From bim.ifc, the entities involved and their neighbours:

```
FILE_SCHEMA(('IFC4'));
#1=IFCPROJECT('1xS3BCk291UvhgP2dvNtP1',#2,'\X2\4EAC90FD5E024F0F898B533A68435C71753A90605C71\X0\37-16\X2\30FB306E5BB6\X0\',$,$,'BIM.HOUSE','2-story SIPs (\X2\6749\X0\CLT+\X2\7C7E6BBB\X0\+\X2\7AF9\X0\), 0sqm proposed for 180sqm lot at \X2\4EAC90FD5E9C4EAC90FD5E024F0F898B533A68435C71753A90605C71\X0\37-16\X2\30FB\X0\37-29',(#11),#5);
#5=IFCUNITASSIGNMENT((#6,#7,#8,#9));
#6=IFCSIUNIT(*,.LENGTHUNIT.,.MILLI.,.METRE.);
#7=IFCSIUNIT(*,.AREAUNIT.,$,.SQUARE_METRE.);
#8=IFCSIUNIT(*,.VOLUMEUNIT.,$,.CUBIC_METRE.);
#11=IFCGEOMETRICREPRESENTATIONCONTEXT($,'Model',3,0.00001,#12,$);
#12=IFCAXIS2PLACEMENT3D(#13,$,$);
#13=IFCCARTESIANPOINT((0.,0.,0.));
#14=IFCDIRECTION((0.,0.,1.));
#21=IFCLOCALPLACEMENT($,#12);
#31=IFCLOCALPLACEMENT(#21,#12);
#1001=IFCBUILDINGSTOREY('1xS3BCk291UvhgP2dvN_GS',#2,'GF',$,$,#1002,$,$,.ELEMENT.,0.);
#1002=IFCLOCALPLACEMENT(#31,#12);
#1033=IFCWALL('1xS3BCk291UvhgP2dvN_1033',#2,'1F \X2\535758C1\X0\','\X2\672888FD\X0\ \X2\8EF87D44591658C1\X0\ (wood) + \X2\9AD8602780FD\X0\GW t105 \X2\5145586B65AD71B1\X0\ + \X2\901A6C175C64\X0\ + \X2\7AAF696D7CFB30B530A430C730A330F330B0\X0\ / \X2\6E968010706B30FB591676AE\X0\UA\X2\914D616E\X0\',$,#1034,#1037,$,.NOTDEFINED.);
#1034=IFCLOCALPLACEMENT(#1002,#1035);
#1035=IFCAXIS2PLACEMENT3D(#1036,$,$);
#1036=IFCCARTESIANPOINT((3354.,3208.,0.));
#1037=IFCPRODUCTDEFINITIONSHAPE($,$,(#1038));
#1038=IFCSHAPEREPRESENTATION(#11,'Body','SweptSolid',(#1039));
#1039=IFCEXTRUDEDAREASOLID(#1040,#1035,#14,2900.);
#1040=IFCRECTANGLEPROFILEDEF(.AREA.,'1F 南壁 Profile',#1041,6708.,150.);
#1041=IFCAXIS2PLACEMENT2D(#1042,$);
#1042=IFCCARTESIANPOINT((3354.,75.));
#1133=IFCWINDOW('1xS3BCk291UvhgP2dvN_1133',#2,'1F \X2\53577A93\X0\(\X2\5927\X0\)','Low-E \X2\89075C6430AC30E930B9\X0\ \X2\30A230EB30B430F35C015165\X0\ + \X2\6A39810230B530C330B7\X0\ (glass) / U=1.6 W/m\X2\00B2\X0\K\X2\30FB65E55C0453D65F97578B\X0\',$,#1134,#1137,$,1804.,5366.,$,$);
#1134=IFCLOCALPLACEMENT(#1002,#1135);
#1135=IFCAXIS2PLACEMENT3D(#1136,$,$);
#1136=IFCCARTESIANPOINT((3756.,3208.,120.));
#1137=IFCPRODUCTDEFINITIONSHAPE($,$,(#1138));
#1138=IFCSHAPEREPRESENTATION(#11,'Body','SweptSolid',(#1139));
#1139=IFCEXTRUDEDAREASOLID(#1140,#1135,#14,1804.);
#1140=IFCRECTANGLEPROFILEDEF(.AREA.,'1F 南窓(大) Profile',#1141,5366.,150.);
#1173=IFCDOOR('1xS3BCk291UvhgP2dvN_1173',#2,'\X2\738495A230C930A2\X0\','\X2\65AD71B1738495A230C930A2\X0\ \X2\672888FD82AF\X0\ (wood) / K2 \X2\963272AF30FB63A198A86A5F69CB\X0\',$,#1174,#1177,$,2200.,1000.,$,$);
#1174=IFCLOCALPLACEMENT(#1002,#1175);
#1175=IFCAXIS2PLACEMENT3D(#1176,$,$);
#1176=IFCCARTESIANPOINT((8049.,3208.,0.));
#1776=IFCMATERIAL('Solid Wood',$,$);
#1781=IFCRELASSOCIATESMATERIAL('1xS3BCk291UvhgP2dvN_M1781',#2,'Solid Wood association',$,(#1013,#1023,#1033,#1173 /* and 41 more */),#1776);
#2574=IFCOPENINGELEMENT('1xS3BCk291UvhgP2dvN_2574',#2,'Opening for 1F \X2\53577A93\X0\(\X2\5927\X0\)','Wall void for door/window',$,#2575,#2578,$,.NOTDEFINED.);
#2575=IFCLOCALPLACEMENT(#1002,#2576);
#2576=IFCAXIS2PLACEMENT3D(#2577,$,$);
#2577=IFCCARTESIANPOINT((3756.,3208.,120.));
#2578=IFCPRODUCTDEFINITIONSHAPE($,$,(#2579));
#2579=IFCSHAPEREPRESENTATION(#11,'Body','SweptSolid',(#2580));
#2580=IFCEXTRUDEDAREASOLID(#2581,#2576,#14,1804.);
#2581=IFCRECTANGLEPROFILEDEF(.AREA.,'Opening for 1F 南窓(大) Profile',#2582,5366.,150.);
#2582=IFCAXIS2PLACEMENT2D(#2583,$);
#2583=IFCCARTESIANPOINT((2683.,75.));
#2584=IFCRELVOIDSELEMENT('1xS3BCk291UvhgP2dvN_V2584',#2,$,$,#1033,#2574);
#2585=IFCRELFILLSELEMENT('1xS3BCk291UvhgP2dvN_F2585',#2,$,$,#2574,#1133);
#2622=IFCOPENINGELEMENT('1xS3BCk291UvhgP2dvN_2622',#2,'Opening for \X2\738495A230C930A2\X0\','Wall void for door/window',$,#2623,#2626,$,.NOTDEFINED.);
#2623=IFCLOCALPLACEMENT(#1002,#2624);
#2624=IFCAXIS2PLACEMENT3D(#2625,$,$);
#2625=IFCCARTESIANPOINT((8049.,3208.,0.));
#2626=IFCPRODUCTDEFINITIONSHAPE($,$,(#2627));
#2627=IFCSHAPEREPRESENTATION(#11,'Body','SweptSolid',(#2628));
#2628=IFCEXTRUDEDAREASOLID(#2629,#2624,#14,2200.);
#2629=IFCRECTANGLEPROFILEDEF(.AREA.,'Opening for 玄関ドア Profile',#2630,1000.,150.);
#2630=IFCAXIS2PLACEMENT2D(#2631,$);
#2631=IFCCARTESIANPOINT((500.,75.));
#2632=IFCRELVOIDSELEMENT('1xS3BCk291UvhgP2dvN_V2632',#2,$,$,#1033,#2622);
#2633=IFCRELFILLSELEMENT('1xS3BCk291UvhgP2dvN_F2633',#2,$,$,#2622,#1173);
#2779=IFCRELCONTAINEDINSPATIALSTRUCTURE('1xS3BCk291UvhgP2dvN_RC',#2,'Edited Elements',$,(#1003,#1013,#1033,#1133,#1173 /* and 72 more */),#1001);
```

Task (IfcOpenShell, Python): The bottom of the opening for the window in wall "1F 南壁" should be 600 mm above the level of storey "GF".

```python
import numpy as np
import ifcopenshell
import ifcopenshell.api.geometry
import ifcopenshell.geom
import ifcopenshell.util.element
import ifcopenshell.util.placement
import ifcopenshell.util.shape
import ifcopenshell.util.unit

model = ifcopenshell.open("bim.ifc")
unit_scale = ifcopenshell.util.unit.calculate_unit_scale(model)

window = model.by_guid("1xS3BCk291UvhgP2dvN_1133")
opening = window.FillsVoids[0].RelatingOpeningElement
storey = ifcopenshell.util.element.get_container(window, ifc_class="IfcBuildingStorey")
level = ifcopenshell.util.placement.get_local_placement(storey.ObjectPlacement)[2, 3]

# The opening's origin need not be at the sill, so measure its lowest point.
shape = ifcopenshell.geom.create_shape(ifcopenshell.geom.settings(), opening)
bottom = ifcopenshell.util.shape.get_shape_bottom_elevation(shape, shape.geometry) / unit_scale
dz = level + 0.6 / unit_scale - bottom

shift = np.array([0.0, 0.0, dz])
# The window is not placed relative to its opening, so move both.
for product in (opening, window):
    matrix = ifcopenshell.util.placement.get_local_placement(product.ObjectPlacement)
    matrix[:3, 3] += shift
    ifcopenshell.api.geometry.edit_object_placement(model, product=product, matrix=matrix, is_si=False)

print(f"moved by {dz * unit_scale:+.3f} m")

model.write("bim_updated.ifc")
```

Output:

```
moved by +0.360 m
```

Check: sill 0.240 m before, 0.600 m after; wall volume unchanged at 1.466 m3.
